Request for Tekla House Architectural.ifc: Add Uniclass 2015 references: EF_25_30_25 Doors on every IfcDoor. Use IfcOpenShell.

First a look at what the model holds.

```python
import ifcopenshell

model = ifcopenshell.open("Tekla House Architectural.ifc")
print(model.schema)
print("classifications:", [c.Name for c in model.by_type("IfcClassification")])
for ifc_class in ("IfcDoor", "IfcRoof", "IfcStair", "IfcWall", "IfcWindow"):
    print(ifc_class, len(model.by_type(ifc_class)))
```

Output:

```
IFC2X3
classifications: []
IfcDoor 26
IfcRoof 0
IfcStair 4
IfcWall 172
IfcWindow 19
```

```python
import ifcopenshell
import ifcopenshell.api.classification

model = ifcopenshell.open("Tekla House Architectural.ifc")

# IFC2X3 requires Source and Edition and has no link from the project to the system.
system = model.create_entity("IfcClassification", Source="NBS", Edition="2015", Name="Uniclass 2015")

codes = {
    "IfcDoor": ("EF_25_30_25", "Doors"),
}
for ifc_class, (code, name) in codes.items():
    products = model.by_type(ifc_class)
    ifcopenshell.api.classification.add_reference(
        model, products=products, classification=system, identification=code, name=name
    )
    print(code, len(products))

model.write("Tekla House Architectural_edited.ifc")
```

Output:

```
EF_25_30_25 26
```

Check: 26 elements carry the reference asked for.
